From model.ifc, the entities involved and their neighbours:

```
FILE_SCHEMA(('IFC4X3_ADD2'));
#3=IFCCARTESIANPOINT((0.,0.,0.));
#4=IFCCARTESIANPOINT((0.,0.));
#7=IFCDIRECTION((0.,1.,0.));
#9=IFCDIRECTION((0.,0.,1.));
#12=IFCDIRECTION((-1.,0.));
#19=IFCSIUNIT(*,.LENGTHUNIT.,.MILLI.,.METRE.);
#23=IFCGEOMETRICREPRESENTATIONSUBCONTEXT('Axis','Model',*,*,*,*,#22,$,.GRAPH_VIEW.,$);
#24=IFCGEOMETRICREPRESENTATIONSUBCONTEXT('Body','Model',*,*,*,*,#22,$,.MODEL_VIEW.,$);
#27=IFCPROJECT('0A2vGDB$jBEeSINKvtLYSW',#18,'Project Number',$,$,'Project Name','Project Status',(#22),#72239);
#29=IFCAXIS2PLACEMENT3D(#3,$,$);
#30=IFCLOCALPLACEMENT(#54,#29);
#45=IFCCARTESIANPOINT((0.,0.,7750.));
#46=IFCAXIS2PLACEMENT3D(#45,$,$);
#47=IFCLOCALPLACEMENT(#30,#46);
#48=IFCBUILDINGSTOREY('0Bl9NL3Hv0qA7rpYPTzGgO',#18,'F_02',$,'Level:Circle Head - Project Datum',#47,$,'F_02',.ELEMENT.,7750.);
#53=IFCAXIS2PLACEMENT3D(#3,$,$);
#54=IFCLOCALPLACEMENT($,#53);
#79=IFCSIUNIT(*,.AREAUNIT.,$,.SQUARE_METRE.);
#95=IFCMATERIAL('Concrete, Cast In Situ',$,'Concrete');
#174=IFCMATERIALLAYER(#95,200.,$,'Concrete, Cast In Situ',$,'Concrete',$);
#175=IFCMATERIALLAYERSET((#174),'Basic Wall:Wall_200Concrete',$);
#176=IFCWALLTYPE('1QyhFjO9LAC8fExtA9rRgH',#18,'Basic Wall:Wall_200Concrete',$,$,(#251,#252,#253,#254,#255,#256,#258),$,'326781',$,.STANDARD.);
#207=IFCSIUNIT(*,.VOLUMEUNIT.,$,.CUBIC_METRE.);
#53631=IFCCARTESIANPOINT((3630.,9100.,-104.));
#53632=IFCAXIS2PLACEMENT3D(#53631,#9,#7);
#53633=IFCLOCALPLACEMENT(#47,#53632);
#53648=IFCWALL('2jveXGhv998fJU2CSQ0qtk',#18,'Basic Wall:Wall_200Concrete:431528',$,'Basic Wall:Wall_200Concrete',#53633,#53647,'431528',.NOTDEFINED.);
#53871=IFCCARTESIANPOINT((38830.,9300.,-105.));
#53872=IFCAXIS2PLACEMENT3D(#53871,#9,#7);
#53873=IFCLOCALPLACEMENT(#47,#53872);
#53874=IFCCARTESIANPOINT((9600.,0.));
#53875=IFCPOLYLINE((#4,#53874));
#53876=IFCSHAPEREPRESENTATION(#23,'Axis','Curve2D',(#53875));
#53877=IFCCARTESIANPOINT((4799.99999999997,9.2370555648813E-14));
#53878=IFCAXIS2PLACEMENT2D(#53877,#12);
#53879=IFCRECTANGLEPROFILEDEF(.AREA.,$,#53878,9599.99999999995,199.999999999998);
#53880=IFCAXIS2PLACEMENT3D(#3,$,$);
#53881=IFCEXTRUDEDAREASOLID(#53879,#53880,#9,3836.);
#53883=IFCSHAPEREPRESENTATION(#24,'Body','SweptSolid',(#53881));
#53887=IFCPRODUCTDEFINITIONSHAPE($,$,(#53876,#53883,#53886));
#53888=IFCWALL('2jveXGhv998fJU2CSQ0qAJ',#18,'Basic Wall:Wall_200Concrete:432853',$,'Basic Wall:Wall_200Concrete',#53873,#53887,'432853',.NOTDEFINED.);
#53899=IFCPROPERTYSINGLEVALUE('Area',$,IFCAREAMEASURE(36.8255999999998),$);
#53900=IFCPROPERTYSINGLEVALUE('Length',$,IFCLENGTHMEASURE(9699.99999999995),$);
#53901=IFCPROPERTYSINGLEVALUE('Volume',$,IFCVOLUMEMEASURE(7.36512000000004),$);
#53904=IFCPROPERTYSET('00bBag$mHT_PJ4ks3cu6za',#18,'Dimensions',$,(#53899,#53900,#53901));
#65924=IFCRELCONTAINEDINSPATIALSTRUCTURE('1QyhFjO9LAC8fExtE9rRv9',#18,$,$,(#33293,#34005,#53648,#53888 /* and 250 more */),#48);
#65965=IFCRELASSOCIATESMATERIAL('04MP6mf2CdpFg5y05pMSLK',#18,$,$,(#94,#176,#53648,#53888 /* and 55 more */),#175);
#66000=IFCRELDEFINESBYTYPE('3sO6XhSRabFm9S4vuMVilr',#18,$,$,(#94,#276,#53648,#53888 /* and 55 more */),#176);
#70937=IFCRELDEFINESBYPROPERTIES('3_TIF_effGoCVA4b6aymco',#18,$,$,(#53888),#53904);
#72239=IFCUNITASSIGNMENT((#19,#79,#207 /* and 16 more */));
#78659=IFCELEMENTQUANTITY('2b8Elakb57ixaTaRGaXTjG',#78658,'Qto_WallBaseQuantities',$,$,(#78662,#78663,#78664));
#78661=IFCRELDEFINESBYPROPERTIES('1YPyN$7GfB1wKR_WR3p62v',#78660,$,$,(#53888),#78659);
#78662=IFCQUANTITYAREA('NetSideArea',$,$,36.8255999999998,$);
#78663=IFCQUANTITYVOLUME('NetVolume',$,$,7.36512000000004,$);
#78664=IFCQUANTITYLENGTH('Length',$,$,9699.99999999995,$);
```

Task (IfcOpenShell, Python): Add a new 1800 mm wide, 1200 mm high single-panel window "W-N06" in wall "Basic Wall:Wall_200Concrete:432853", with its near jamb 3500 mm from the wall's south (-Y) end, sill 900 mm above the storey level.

```python
import numpy as np
import ifcopenshell
import ifcopenshell.api.feature
import ifcopenshell.api.geometry
import ifcopenshell.api.pset
import ifcopenshell.api.root
import ifcopenshell.api.spatial
import ifcopenshell.geom
import ifcopenshell.util.element
import ifcopenshell.util.placement
import ifcopenshell.util.representation
import ifcopenshell.util.shape
import ifcopenshell.util.unit

model = ifcopenshell.open("model.ifc")
unit_scale = ifcopenshell.util.unit.calculate_unit_scale(model)
area_scale = ifcopenshell.util.unit.calculate_unit_scale(model, "AREAUNIT")
volume_scale = ifcopenshell.util.unit.calculate_unit_scale(model, "VOLUMEUNIT")
settings = ifcopenshell.geom.settings()


def volume(element):
    """Net volume in cubic metres, openings subtracted."""
    shape = ifcopenshell.geom.create_shape(settings, element)
    return ifcopenshell.util.shape.get_volume(shape.geometry)


wall = model.by_guid("2jveXGhv998fJU2CSQ0qAJ")
storey = ifcopenshell.util.element.get_container(wall, ifc_class="IfcBuildingStorey")
context = ifcopenshell.util.representation.get_context(model, "Model", "Body", "MODEL_VIEW")
before = volume(wall)

width, height, from_end, sill = 1.8, 1.2, 3.5, 0.9  # metres

# The wall runs along its own X axis, and the end named is its -X end.
wall_shape = ifcopenshell.geom.create_shape(settings, wall)
x, y, z = ifcopenshell.util.shape.get_vertices(wall_shape.geometry).T
start = x.min() + from_end
face, thickness = float(y.min()), float(y.max() - y.min())
wall_matrix = ifcopenshell.util.placement.get_local_placement(wall.ObjectPlacement)
level = ifcopenshell.util.placement.get_local_placement(storey.ObjectPlacement)[2, 3]


def in_wall(x, y):
    """Placement at x, y metres in the wall's axes, at sill height."""
    matrix = wall_matrix.copy()
    matrix[:, 3] = wall_matrix @ np.array([x / unit_scale, y / unit_scale, 0.0, 1.0])
    matrix[2, 3] = level + sill / unit_scale
    return matrix


# Opening: a box that overshoots both wall faces by 50 mm.
opening = ifcopenshell.api.root.create_entity(model, ifc_class="IfcOpeningElement", predefined_type="OPENING")
box = ifcopenshell.api.geometry.add_wall_representation(
    model, context=context, length=width, height=height, thickness=thickness + 0.1
)
ifcopenshell.api.geometry.assign_representation(model, product=opening, representation=box)
ifcopenshell.api.geometry.edit_object_placement(model, product=opening, matrix=in_wall(start, face - 0.05), is_si=False)
ifcopenshell.api.feature.add_feature(model, feature=opening, element=wall)

window = ifcopenshell.api.root.create_entity(model, ifc_class="IfcWindow", name="W-N06", predefined_type="WINDOW")
window.OverallWidth, window.OverallHeight = width / unit_scale, height / unit_scale
window.PartitioningType = "SINGLE_PANEL"
body = ifcopenshell.api.geometry.add_window_representation(
    model,
    context=context,
    overall_width=window.OverallWidth,
    overall_height=window.OverallHeight,
    partition_type="SINGLE_PANEL",
)
ifcopenshell.api.geometry.assign_representation(model, product=window, representation=body)
ifcopenshell.api.spatial.assign_container(model, products=[window], relating_structure=storey)
ifcopenshell.api.feature.add_filling(model, opening=opening, element=window)

# Centre the window in the wall's thickness.
ifcopenshell.api.geometry.edit_object_placement(model, product=window, matrix=in_wall(start, face), is_si=False)
window_shape = ifcopenshell.geom.create_shape(settings, window)
depth = ifcopenshell.util.shape.get_vertices(window_shape.geometry)[:, 1]
offset = face + thickness / 2 - (depth.min() + depth.max()) / 2
ifcopenshell.api.geometry.edit_object_placement(model, product=window, matrix=in_wall(start, offset), is_si=False)

after = volume(wall)

# Update the wall's stored quantities.
pset = model.by_id(ifcopenshell.util.element.get_pset(wall, "Dimensions", should_inherit=False)["id"])
ifcopenshell.api.pset.edit_pset(model, pset=pset, properties={
    "Area": model.create_entity("IfcAreaMeasure", after / thickness / area_scale),
    "Volume": model.create_entity("IfcVolumeMeasure", after / volume_scale),
})
qto = model.by_id(ifcopenshell.util.element.get_pset(wall, "Qto_WallBaseQuantities", should_inherit=False)["id"])
ifcopenshell.api.pset.edit_qto(model, qto=qto, properties={
    "NetSideArea": after / thickness / area_scale,
    "NetVolume": after / volume_scale,
})

print(f"wall volume {before:.3f} -> {after:.3f} m3")

model.write("model_updated.ifc")
```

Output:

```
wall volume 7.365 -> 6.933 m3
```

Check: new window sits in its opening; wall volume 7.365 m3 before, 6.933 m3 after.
